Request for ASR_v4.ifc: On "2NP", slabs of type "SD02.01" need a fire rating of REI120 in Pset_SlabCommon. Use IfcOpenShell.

First a look at what the model holds.

```python
import ifcopenshell
import ifcopenshell.util.element

model = ifcopenshell.open("ASR_v4.ifc")
print(model.schema)
storey = next(s for s in model.by_type("IfcBuildingStorey") if s.Name == "2NP")
slabs = [e for e in ifcopenshell.util.element.get_decomposition(storey) if e.is_a("IfcSlab")]
seen = {}
for e in slabs:
    element_type = ifcopenshell.util.element.get_type(e)
    key = (element_type.Name if element_type != e and element_type else None, ifcopenshell.util.element.get_pset(e, "Pset_SlabCommon", "FireRating"))
    seen[key] = seen.get(key, 0) + 1
for (name, value), count in sorted(seen.items(), key=str):
    print(count, "x", name, "|", value)
```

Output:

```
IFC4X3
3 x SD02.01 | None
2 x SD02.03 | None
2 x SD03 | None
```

```python
import ifcopenshell
import ifcopenshell.api.pset
import ifcopenshell.util.element

model = ifcopenshell.open("ASR_v4.ifc")

storey = next(s for s in model.by_type("IfcBuildingStorey") if s.Name == "2NP")
slabs = [e for e in ifcopenshell.util.element.get_decomposition(storey) if e.is_a("IfcSlab")]

count = 0
for e in slabs:
    element_type = ifcopenshell.util.element.get_type(e)
    if element_type in (None, e) or element_type.Name != "SD02.01":
        continue
    # add_pset returns the element's existing set when there is one.
    pset = ifcopenshell.api.pset.add_pset(model, product=e, name="Pset_SlabCommon")
    ifcopenshell.api.pset.edit_pset(model, pset=pset, properties={"FireRating": "REI120"})
    count += 1

print(count, "slabs updated")

model.write("ASR_v4_updated.ifc")
```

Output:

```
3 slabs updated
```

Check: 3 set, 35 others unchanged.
